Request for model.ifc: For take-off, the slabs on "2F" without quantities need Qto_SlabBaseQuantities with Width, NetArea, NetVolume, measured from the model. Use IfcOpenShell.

First a look at what the model holds.

```python
import ifcopenshell
import ifcopenshell.util.element
import ifcopenshell.util.unit

model = ifcopenshell.open("model.ifc")
print(model.schema)
for unit_type in ("LENGTHUNIT", "AREAUNIT", "VOLUMEUNIT"):
    print(unit_type, ifcopenshell.util.unit.calculate_unit_scale(model, unit_type))
storey = next(s for s in model.by_type("IfcBuildingStorey") if s.Name == "2F")
slabs = [e for e in ifcopenshell.util.element.get_decomposition(storey) if e.is_a("IfcSlab")]
for e in sorted(slabs, key=lambda e: e.id()):
    print(e.id(), e.is_a(), e.Name, list(ifcopenshell.util.element.get_psets(e, qtos_only=True)), sep=" | ")
```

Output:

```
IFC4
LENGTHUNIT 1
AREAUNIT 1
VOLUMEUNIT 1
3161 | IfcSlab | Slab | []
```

```python
import ifcopenshell
import ifcopenshell.api.pset
import ifcopenshell.geom
import ifcopenshell.util.element
import ifcopenshell.util.shape
import ifcopenshell.util.unit

model = ifcopenshell.open("model.ifc")
unit_scale = ifcopenshell.util.unit.calculate_unit_scale(model)
area_scale = ifcopenshell.util.unit.calculate_unit_scale(model, "AREAUNIT")
volume_scale = ifcopenshell.util.unit.calculate_unit_scale(model, "VOLUMEUNIT")
settings = ifcopenshell.geom.settings()

storey = next(s for s in model.by_type("IfcBuildingStorey") if s.Name == "2F")
slabs = [e for e in ifcopenshell.util.element.get_decomposition(storey) if e.is_a("IfcSlab")]

for e in sorted(slabs, key=lambda e: e.id()):
    if ifcopenshell.util.element.get_psets(e, qtos_only=True, should_inherit=False):
        continue
    # Geometry comes back in metres, in the element's own axes.
    shape = ifcopenshell.geom.create_shape(settings, e)
    values = {
        "Width": ifcopenshell.util.shape.get_z(shape.geometry) / unit_scale,
        "NetArea": ifcopenshell.util.shape.get_footprint_area(shape.geometry) / area_scale,
        "NetVolume": ifcopenshell.util.shape.get_volume(shape.geometry) / volume_scale,
    }
    qto = ifcopenshell.api.pset.add_qto(model, product=e, name="Qto_SlabBaseQuantities")
    ifcopenshell.api.pset.edit_qto(model, qto=qto, properties=values)
    print(e.id(), {k: round(v, 3) for k, v in values.items()})

model.write("model_rev.ifc")
```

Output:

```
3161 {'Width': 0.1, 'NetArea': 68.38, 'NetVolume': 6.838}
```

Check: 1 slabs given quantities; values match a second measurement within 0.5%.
